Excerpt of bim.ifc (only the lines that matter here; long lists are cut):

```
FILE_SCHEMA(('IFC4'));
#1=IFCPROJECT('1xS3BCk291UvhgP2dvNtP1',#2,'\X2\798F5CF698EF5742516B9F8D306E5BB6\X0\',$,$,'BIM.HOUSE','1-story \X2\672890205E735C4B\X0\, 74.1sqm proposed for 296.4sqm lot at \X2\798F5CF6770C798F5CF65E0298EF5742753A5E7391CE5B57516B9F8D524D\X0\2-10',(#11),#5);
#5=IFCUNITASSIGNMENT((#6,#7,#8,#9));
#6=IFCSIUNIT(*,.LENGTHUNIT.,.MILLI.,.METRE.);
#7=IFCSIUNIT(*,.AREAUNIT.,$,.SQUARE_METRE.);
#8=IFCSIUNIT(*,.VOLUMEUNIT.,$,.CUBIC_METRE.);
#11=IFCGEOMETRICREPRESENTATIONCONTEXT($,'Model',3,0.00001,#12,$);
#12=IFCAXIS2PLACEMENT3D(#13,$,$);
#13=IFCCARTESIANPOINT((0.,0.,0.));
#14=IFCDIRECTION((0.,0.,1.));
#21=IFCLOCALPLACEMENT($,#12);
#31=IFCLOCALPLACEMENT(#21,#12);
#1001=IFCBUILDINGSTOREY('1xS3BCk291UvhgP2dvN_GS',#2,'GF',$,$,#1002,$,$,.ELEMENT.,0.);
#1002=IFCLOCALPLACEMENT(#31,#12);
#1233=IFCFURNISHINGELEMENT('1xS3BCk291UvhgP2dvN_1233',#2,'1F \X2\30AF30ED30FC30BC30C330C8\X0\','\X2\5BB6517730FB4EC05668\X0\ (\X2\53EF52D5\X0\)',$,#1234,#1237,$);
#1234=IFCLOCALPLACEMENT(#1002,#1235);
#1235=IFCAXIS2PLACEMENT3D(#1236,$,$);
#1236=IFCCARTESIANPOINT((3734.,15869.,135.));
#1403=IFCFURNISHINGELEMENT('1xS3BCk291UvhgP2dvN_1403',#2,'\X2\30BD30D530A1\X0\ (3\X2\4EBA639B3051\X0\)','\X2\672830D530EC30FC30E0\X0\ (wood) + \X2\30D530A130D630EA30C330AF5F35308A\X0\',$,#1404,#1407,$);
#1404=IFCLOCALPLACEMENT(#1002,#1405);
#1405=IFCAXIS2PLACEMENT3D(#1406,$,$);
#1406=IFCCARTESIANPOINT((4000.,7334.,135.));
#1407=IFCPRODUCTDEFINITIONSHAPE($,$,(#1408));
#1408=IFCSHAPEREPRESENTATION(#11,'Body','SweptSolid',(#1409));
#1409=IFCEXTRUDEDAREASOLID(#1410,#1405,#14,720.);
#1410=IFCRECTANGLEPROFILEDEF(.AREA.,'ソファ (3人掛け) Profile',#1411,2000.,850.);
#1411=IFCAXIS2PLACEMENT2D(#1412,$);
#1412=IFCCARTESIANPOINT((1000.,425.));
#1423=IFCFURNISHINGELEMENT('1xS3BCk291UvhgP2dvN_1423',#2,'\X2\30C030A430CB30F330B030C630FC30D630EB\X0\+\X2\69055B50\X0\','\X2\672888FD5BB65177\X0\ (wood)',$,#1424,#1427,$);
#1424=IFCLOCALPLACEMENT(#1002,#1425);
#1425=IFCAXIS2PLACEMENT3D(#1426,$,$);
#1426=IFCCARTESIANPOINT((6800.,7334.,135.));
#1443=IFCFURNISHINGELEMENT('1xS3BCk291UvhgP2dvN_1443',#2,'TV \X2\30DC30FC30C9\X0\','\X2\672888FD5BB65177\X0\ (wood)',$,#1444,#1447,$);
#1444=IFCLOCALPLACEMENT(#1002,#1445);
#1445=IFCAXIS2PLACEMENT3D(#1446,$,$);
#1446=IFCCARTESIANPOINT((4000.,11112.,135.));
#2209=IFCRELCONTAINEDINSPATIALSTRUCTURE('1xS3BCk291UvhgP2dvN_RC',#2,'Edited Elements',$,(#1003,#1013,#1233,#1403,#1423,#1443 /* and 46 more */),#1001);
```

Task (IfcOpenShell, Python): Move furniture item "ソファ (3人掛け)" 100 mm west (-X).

```python
import ifcopenshell
import ifcopenshell.api.geometry
import ifcopenshell.util.placement
import ifcopenshell.util.unit

model = ifcopenshell.open("bim.ifc")
unit_scale = ifcopenshell.util.unit.calculate_unit_scale(model)

item = model.by_guid("1xS3BCk291UvhgP2dvN_1403")
matrix = ifcopenshell.util.placement.get_local_placement(item.ObjectPlacement)
matrix[0, 3] -= 0.1 / unit_scale
ifcopenshell.api.geometry.edit_object_placement(model, product=item, matrix=matrix, is_si=False)

print(ifcopenshell.util.placement.get_local_placement(item.ObjectPlacement).round(3) + 0.0)

model.write("bim_v2.ifc")
```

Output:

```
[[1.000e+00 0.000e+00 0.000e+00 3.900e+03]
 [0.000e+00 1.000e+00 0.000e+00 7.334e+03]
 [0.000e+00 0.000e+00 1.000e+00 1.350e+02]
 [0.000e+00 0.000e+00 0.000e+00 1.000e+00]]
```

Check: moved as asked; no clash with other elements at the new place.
